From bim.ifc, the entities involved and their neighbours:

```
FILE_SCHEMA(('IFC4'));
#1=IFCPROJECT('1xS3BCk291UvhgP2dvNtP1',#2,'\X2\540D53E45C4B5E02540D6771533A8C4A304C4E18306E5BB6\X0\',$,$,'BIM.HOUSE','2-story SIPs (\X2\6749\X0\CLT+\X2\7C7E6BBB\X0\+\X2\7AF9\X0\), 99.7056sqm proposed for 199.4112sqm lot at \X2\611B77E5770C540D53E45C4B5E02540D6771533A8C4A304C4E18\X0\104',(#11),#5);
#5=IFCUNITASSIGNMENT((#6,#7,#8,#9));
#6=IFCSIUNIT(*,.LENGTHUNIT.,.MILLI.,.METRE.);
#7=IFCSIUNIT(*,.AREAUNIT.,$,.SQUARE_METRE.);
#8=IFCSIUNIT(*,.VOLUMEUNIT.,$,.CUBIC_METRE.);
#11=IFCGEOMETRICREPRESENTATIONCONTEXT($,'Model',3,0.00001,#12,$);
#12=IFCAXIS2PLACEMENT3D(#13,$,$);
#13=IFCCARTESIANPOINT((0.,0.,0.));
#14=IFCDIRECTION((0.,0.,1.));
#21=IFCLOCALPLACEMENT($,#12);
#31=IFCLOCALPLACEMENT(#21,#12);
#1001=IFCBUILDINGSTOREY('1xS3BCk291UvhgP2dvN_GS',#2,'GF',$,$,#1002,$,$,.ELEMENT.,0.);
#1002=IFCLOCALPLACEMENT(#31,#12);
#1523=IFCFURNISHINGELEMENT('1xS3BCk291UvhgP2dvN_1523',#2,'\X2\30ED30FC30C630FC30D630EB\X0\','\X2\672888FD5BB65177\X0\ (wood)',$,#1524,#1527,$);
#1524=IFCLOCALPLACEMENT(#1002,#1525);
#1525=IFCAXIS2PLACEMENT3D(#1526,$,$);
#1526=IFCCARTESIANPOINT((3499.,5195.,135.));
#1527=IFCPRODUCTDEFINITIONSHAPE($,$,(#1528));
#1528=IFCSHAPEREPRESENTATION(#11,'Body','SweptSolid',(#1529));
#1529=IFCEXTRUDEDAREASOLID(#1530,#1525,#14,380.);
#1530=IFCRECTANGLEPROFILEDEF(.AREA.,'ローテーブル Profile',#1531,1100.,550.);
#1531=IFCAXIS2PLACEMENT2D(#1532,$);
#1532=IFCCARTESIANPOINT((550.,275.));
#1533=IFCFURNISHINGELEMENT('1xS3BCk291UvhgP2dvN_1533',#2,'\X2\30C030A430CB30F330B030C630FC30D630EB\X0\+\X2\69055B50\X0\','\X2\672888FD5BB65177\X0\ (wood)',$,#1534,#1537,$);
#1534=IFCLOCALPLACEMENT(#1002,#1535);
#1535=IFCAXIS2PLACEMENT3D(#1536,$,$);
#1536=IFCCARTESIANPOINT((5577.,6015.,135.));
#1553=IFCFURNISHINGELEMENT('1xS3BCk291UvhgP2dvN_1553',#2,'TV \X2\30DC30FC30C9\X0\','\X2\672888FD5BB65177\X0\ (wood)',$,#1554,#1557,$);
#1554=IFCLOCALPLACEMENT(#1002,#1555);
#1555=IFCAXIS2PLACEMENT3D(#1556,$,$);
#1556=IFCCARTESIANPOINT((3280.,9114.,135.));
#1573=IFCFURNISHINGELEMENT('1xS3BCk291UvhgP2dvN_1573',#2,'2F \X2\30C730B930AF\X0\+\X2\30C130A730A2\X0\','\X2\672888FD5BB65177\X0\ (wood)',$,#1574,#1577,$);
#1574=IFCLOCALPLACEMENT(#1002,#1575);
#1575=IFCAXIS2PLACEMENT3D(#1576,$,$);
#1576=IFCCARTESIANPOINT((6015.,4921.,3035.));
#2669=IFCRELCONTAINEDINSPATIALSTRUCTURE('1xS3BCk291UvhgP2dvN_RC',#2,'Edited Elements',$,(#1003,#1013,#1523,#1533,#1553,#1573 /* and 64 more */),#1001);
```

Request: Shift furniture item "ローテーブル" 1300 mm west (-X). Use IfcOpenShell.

```python
import ifcopenshell
import ifcopenshell.api.geometry
import ifcopenshell.util.placement

model = ifcopenshell.open("bim.ifc")

item = model.by_guid("1xS3BCk291UvhgP2dvN_1523")
matrix = ifcopenshell.util.placement.get_local_placement(item.ObjectPlacement)
matrix[0, 3] -= 1300.0
ifcopenshell.api.geometry.edit_object_placement(model, product=item, matrix=matrix, is_si=False)

print(ifcopenshell.util.placement.get_local_placement(item.ObjectPlacement).round(3) + 0.0)

model.write("bim-out.ifc")
```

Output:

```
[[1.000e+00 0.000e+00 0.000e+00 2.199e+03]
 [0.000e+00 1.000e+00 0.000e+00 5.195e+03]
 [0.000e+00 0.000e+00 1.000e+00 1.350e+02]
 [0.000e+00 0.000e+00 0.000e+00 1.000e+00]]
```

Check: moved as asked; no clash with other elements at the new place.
